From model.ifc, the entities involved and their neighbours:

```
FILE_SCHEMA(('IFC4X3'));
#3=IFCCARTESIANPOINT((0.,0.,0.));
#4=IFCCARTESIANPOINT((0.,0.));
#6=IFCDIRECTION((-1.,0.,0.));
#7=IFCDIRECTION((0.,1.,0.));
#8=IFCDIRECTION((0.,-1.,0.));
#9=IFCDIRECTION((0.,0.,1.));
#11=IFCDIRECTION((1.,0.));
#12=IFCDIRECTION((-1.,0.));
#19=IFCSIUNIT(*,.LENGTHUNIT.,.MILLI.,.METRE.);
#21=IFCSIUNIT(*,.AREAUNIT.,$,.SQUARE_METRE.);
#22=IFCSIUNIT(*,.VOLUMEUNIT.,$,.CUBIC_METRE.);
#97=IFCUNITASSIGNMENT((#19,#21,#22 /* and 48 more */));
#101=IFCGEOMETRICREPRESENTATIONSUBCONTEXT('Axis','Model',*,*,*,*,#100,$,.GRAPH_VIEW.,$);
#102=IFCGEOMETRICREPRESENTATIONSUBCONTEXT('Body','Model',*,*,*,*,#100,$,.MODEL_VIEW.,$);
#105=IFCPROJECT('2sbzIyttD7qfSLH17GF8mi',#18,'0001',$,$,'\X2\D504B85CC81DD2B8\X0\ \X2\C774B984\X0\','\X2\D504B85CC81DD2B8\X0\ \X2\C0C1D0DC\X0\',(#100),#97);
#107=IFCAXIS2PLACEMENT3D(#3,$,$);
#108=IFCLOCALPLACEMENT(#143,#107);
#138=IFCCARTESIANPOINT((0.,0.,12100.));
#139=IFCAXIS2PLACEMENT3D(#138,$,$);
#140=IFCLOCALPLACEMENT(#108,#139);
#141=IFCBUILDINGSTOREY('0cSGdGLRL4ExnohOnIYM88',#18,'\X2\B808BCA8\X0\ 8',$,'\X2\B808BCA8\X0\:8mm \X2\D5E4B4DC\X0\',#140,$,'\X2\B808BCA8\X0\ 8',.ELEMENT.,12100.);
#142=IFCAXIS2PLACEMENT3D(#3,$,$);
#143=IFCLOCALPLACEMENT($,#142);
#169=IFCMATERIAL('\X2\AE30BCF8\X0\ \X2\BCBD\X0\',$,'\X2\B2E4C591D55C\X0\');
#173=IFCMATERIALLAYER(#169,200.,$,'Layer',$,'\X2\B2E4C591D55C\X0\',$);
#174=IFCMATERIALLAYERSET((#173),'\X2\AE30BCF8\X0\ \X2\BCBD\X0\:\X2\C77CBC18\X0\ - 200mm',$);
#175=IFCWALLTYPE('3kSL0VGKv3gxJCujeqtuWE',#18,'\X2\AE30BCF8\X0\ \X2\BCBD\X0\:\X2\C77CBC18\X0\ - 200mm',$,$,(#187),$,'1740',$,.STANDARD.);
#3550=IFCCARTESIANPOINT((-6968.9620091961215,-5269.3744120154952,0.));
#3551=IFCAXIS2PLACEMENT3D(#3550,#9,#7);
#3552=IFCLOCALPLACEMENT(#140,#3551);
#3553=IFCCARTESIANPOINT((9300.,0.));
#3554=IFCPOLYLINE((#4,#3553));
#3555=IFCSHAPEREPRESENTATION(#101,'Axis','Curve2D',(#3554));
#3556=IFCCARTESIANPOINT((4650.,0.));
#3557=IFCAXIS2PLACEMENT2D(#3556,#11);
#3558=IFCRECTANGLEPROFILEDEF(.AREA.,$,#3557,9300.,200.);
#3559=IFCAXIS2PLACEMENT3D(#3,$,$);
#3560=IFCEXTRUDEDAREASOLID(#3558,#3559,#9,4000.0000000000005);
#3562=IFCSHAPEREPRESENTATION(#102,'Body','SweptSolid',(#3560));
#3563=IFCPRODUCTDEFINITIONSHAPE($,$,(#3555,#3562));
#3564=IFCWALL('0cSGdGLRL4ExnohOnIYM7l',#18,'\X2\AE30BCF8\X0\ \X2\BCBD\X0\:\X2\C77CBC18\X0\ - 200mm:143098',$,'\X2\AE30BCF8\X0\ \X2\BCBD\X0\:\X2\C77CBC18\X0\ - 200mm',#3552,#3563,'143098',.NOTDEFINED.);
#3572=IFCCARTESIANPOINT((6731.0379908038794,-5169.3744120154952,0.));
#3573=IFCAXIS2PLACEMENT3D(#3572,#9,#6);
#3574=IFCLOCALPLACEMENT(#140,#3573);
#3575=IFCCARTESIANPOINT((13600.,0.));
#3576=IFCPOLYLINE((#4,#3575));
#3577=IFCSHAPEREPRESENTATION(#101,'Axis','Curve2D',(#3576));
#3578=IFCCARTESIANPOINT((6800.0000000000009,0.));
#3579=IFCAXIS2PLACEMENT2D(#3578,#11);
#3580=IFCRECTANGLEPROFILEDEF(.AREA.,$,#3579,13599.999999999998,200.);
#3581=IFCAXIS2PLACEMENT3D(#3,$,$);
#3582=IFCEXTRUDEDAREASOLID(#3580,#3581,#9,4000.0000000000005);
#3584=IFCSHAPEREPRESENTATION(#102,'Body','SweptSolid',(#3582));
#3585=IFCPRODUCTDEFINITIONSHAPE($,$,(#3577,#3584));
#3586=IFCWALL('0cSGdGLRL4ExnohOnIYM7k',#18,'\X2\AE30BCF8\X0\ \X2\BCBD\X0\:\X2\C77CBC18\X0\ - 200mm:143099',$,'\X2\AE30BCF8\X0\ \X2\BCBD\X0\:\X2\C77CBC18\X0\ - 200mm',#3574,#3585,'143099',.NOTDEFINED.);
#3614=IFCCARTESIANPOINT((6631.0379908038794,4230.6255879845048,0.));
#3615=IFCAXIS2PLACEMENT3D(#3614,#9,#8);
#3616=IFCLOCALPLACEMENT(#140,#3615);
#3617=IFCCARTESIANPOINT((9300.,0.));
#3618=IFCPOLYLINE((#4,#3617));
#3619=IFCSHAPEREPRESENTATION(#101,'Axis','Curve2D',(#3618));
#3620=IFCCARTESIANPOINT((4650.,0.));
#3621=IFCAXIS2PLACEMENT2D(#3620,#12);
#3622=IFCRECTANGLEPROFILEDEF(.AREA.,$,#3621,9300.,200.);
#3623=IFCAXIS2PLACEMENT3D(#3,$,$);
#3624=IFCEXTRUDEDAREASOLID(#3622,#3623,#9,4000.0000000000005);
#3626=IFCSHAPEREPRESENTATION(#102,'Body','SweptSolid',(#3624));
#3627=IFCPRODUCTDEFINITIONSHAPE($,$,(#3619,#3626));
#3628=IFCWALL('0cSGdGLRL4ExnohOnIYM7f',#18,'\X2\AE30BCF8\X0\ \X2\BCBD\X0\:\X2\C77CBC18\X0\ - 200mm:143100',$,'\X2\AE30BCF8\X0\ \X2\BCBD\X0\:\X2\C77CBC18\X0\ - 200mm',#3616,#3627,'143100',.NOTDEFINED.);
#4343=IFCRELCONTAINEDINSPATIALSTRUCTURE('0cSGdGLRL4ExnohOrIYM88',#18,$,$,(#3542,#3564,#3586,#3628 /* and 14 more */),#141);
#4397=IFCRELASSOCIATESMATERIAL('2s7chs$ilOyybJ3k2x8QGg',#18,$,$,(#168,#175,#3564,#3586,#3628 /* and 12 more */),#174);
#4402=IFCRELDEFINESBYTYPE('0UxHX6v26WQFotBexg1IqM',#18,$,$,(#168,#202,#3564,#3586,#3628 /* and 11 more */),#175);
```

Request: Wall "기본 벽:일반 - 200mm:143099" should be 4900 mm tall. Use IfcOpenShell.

```python
import ifcopenshell
import ifcopenshell.geom
import ifcopenshell.util.representation
import ifcopenshell.util.shape
import ifcopenshell.util.unit

model = ifcopenshell.open("model.ifc")
unit_scale = ifcopenshell.util.unit.calculate_unit_scale(model)
settings = ifcopenshell.geom.settings()


def volume(element):
    """Net volume in cubic metres, openings subtracted."""
    shape = ifcopenshell.geom.create_shape(settings, element)
    return ifcopenshell.util.shape.get_volume(shape.geometry)


wall = model.by_guid("0cSGdGLRL4ExnohOnIYM7k")
before = volume(wall)

body = ifcopenshell.util.representation.get_representation(wall, "Model", "Body")
solid = body.Items[0]
old_height = solid.Depth
solid.Depth = 4.9 / unit_scale
after = volume(wall)

print(f"height {old_height:g} -> {solid.Depth:g}, volume {before:.3f} -> {after:.3f} m3")

model.write("model_rev.ifc")
```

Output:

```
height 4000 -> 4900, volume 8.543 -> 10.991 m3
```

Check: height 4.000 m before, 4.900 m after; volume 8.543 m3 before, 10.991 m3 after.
